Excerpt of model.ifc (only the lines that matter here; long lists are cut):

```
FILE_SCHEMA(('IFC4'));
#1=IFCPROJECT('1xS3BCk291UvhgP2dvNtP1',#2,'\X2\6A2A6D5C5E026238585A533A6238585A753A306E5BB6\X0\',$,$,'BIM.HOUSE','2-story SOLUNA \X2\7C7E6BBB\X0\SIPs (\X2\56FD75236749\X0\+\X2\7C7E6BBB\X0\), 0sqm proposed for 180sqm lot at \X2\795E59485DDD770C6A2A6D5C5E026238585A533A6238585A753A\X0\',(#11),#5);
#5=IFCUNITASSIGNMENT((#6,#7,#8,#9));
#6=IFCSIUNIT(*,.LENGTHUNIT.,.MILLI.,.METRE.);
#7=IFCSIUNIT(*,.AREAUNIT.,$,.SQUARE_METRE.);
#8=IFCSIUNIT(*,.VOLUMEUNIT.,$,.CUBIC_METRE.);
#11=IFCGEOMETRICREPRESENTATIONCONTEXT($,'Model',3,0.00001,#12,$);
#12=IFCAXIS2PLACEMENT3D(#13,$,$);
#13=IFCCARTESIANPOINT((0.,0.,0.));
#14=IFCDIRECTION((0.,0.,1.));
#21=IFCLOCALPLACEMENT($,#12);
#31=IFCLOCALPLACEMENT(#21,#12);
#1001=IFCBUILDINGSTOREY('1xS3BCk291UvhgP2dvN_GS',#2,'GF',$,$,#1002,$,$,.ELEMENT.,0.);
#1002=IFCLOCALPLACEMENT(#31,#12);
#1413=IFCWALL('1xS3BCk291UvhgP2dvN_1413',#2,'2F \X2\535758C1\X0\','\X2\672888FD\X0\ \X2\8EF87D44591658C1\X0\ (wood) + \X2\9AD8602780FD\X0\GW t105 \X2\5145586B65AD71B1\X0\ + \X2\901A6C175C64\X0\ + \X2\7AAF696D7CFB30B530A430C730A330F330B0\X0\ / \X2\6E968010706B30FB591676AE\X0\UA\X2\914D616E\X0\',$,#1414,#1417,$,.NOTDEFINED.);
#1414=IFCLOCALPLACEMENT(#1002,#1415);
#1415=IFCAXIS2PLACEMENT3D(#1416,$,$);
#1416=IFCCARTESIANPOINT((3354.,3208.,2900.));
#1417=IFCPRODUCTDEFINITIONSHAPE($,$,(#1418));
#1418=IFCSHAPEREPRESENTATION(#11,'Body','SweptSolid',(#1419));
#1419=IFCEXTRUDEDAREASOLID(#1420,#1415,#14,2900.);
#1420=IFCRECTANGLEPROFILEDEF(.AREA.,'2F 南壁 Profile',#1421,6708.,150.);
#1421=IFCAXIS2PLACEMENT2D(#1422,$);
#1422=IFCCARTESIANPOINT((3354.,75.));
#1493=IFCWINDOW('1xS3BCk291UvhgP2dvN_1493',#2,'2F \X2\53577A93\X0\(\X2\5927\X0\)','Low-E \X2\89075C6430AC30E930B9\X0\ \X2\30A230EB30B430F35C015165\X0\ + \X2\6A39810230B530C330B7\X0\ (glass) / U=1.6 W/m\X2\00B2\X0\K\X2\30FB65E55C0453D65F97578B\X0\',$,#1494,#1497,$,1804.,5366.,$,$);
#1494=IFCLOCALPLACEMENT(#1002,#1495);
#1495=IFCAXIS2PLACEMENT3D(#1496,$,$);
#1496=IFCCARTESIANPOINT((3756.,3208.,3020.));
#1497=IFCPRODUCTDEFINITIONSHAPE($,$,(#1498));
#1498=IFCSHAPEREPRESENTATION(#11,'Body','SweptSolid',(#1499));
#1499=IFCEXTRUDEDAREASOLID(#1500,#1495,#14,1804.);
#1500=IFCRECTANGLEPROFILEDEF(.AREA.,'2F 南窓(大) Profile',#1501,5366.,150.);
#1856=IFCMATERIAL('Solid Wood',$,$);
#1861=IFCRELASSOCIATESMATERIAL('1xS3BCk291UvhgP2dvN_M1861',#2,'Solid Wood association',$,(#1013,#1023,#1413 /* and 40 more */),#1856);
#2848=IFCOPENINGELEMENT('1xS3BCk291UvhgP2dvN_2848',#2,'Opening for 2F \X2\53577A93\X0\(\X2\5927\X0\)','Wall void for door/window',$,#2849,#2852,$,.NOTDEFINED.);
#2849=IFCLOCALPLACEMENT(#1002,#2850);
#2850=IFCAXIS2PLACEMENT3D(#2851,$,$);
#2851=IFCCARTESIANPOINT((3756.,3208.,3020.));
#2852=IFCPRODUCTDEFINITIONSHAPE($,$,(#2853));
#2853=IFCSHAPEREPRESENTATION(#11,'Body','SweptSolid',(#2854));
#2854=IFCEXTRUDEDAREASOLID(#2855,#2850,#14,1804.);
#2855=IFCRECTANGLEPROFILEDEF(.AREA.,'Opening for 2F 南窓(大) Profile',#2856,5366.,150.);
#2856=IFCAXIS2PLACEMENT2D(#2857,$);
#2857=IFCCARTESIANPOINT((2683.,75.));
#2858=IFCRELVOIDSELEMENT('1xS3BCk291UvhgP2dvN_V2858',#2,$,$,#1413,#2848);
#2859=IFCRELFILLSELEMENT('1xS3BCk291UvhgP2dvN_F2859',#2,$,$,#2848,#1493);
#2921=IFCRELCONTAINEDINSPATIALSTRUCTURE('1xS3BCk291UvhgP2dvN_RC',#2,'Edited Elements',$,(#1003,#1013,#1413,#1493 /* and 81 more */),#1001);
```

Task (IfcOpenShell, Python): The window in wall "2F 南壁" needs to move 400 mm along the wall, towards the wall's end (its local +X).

```python
import ifcopenshell
import ifcopenshell.api.geometry
import ifcopenshell.util.placement

model = ifcopenshell.open("model.ifc")

window = model.by_guid("1xS3BCk291UvhgP2dvN_1493")
opening = window.FillsVoids[0].RelatingOpeningElement
wall = opening.VoidsElements[0].RelatingBuildingElement

wall_matrix = ifcopenshell.util.placement.get_local_placement(wall.ObjectPlacement)
shift = wall_matrix[:3, 0] * 400.0
before = ifcopenshell.util.placement.get_local_placement(window.ObjectPlacement)[:3, 3].copy()

# The window is not placed relative to its opening, so move both.
for product in (opening, window):
    matrix = ifcopenshell.util.placement.get_local_placement(product.ObjectPlacement)
    matrix[:3, 3] += shift
    ifcopenshell.api.geometry.edit_object_placement(model, product=product, matrix=matrix, is_si=False)

after = ifcopenshell.util.placement.get_local_placement(window.ObjectPlacement)[:3, 3]
print("window moved by", (after - before).round(3) + 0.0)

model.write("model_v2.ifc")
```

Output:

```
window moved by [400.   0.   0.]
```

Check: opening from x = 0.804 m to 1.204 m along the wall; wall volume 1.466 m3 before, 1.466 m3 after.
